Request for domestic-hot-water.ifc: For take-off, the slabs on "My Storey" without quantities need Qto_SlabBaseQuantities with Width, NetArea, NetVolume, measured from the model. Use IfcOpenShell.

First a look at what the model holds.

```python
import ifcopenshell
import ifcopenshell.util.element
import ifcopenshell.util.unit

model = ifcopenshell.open("domestic-hot-water.ifc")
print(model.schema)
for unit_type in ("LENGTHUNIT", "AREAUNIT", "VOLUMEUNIT"):
    print(unit_type, ifcopenshell.util.unit.calculate_unit_scale(model, unit_type))
storey = next(s for s in model.by_type("IfcBuildingStorey") if s.Name == "My Storey")
slabs = [e for e in ifcopenshell.util.element.get_decomposition(storey) if e.is_a("IfcSlab")]
for e in sorted(slabs, key=lambda e: e.id()):
    print(e.id(), e.is_a(), e.Name, list(ifcopenshell.util.element.get_psets(e, qtos_only=True)), sep=" | ")
```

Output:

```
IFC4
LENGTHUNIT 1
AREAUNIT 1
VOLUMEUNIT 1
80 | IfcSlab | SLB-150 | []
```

```python
import ifcopenshell
import ifcopenshell.api.pset
import ifcopenshell.geom
import ifcopenshell.util.element
import ifcopenshell.util.shape
import ifcopenshell.util.unit

model = ifcopenshell.open("domestic-hot-water.ifc")
unit_scale = ifcopenshell.util.unit.calculate_unit_scale(model)
area_scale = ifcopenshell.util.unit.calculate_unit_scale(model, "AREAUNIT")
volume_scale = ifcopenshell.util.unit.calculate_unit_scale(model, "VOLUMEUNIT")
settings = ifcopenshell.geom.settings()

storey = next(s for s in model.by_type("IfcBuildingStorey") if s.Name == "My Storey")
slabs = [e for e in ifcopenshell.util.element.get_decomposition(storey) if e.is_a("IfcSlab")]

for e in sorted(slabs, key=lambda e: e.id()):
    if ifcopenshell.util.element.get_psets(e, qtos_only=True, should_inherit=False):
        continue
    # Geometry comes back in metres, in the element's own axes.
    shape = ifcopenshell.geom.create_shape(settings, e)
    values = {
        "Width": ifcopenshell.util.shape.get_z(shape.geometry) / unit_scale,
        "NetArea": ifcopenshell.util.shape.get_footprint_area(shape.geometry) / area_scale,
        "NetVolume": ifcopenshell.util.shape.get_volume(shape.geometry) / volume_scale,
    }
    qto = ifcopenshell.api.pset.add_qto(model, product=e, name="Qto_SlabBaseQuantities")
    ifcopenshell.api.pset.edit_qto(model, qto=qto, properties=values)
    print(e.id(), {k: round(v, 3) for k, v in values.items()})

model.write("domestic-hot-water_updated.ifc")
```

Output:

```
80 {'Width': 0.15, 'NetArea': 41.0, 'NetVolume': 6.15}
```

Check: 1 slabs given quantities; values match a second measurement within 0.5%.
